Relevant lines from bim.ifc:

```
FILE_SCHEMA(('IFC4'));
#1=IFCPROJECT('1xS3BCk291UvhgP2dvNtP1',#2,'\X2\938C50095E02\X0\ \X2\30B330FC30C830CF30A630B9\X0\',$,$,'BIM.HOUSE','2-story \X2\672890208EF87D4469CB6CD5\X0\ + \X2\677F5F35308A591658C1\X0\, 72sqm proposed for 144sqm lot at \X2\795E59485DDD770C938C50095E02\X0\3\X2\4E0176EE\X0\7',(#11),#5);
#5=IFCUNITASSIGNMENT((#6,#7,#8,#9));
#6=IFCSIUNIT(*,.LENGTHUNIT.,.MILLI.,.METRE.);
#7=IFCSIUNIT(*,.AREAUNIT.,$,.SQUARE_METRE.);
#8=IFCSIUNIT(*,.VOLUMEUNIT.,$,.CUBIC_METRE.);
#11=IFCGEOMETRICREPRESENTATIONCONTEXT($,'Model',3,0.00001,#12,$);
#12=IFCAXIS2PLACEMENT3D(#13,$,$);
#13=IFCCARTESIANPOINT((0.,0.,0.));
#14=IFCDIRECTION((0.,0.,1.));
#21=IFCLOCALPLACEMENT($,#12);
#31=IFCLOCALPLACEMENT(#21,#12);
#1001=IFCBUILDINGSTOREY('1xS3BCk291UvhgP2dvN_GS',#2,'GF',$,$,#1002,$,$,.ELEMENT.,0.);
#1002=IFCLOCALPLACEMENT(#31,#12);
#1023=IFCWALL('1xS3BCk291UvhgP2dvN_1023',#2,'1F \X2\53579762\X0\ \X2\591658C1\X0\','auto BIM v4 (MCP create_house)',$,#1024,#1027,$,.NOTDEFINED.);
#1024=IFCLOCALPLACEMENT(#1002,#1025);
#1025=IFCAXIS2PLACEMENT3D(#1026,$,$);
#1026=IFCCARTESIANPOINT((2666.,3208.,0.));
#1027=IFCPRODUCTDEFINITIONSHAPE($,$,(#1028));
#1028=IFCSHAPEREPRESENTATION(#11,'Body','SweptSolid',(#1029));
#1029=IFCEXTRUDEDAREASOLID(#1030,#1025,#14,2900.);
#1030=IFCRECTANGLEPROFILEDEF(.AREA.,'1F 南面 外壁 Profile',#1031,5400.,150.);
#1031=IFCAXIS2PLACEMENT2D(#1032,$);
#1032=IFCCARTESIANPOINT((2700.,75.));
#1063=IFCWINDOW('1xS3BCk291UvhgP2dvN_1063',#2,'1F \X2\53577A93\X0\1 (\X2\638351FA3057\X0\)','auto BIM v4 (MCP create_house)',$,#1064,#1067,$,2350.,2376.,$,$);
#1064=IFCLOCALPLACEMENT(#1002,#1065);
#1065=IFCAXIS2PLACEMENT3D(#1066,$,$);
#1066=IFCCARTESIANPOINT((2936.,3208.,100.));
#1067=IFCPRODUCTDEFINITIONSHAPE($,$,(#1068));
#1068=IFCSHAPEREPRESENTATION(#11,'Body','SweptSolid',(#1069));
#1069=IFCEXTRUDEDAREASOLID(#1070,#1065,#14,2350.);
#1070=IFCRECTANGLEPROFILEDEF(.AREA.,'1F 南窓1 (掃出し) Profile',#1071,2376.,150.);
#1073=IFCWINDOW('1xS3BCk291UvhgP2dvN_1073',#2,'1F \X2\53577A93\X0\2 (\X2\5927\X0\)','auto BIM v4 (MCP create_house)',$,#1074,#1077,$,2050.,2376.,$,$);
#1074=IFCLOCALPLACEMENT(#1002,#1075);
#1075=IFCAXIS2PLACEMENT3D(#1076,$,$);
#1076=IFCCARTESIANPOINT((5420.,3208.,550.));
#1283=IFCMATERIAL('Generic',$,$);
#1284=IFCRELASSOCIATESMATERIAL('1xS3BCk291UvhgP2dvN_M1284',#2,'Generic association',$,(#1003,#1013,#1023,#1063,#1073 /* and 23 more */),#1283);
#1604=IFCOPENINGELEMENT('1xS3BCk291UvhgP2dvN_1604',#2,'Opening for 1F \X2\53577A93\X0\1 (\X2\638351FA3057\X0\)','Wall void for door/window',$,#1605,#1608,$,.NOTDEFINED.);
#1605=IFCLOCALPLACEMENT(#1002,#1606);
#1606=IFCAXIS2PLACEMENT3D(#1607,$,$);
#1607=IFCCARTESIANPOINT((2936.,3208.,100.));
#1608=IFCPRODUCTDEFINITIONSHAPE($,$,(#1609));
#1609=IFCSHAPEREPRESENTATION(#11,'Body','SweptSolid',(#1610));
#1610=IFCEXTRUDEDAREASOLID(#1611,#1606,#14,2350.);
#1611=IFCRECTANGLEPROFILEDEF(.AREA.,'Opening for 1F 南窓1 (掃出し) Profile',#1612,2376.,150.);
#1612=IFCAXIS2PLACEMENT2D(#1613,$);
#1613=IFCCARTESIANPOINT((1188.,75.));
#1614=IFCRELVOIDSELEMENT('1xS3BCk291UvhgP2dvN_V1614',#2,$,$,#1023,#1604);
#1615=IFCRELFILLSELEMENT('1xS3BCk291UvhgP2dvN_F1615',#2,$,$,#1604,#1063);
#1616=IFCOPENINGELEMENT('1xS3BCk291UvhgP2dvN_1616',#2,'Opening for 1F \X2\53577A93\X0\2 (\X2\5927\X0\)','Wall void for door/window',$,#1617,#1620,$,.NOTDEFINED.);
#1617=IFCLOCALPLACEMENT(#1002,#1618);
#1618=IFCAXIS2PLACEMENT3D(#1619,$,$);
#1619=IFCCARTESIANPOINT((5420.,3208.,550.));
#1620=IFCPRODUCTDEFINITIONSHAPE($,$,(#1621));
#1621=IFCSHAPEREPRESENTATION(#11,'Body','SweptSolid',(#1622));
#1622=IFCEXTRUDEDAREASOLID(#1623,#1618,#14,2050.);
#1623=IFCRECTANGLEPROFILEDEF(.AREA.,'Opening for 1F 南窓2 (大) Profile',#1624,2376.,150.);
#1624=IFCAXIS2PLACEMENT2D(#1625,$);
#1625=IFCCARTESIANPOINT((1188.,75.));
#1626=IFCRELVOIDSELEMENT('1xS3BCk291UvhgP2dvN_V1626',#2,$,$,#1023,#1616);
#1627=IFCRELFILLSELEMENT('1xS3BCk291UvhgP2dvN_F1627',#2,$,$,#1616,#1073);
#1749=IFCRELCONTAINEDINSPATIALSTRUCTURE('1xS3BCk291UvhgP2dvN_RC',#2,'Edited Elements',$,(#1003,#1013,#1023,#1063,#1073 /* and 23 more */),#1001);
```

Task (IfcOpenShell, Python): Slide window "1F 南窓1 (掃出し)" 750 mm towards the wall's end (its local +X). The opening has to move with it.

```python
import ifcopenshell
import ifcopenshell.api.geometry
import ifcopenshell.util.placement

model = ifcopenshell.open("bim.ifc")

window = model.by_id(1063)
opening = window.FillsVoids[0].RelatingOpeningElement
wall = opening.VoidsElements[0].RelatingBuildingElement

wall_matrix = ifcopenshell.util.placement.get_local_placement(wall.ObjectPlacement)
shift = wall_matrix[:3, 0] * 750.0
before = ifcopenshell.util.placement.get_local_placement(window.ObjectPlacement)[:3, 3].copy()

# The window is not placed relative to its opening, so move both.
for product in (opening, window):
    matrix = ifcopenshell.util.placement.get_local_placement(product.ObjectPlacement)
    matrix[:3, 3] += shift
    ifcopenshell.api.geometry.edit_object_placement(model, product=product, matrix=matrix, is_si=False)

after = ifcopenshell.util.placement.get_local_placement(window.ObjectPlacement)[:3, 3]
print("window moved by", (after - before).round(3) + 0.0)

model.write("bim_edited.ifc")
```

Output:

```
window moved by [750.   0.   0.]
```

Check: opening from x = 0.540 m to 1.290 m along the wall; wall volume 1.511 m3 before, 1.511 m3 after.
